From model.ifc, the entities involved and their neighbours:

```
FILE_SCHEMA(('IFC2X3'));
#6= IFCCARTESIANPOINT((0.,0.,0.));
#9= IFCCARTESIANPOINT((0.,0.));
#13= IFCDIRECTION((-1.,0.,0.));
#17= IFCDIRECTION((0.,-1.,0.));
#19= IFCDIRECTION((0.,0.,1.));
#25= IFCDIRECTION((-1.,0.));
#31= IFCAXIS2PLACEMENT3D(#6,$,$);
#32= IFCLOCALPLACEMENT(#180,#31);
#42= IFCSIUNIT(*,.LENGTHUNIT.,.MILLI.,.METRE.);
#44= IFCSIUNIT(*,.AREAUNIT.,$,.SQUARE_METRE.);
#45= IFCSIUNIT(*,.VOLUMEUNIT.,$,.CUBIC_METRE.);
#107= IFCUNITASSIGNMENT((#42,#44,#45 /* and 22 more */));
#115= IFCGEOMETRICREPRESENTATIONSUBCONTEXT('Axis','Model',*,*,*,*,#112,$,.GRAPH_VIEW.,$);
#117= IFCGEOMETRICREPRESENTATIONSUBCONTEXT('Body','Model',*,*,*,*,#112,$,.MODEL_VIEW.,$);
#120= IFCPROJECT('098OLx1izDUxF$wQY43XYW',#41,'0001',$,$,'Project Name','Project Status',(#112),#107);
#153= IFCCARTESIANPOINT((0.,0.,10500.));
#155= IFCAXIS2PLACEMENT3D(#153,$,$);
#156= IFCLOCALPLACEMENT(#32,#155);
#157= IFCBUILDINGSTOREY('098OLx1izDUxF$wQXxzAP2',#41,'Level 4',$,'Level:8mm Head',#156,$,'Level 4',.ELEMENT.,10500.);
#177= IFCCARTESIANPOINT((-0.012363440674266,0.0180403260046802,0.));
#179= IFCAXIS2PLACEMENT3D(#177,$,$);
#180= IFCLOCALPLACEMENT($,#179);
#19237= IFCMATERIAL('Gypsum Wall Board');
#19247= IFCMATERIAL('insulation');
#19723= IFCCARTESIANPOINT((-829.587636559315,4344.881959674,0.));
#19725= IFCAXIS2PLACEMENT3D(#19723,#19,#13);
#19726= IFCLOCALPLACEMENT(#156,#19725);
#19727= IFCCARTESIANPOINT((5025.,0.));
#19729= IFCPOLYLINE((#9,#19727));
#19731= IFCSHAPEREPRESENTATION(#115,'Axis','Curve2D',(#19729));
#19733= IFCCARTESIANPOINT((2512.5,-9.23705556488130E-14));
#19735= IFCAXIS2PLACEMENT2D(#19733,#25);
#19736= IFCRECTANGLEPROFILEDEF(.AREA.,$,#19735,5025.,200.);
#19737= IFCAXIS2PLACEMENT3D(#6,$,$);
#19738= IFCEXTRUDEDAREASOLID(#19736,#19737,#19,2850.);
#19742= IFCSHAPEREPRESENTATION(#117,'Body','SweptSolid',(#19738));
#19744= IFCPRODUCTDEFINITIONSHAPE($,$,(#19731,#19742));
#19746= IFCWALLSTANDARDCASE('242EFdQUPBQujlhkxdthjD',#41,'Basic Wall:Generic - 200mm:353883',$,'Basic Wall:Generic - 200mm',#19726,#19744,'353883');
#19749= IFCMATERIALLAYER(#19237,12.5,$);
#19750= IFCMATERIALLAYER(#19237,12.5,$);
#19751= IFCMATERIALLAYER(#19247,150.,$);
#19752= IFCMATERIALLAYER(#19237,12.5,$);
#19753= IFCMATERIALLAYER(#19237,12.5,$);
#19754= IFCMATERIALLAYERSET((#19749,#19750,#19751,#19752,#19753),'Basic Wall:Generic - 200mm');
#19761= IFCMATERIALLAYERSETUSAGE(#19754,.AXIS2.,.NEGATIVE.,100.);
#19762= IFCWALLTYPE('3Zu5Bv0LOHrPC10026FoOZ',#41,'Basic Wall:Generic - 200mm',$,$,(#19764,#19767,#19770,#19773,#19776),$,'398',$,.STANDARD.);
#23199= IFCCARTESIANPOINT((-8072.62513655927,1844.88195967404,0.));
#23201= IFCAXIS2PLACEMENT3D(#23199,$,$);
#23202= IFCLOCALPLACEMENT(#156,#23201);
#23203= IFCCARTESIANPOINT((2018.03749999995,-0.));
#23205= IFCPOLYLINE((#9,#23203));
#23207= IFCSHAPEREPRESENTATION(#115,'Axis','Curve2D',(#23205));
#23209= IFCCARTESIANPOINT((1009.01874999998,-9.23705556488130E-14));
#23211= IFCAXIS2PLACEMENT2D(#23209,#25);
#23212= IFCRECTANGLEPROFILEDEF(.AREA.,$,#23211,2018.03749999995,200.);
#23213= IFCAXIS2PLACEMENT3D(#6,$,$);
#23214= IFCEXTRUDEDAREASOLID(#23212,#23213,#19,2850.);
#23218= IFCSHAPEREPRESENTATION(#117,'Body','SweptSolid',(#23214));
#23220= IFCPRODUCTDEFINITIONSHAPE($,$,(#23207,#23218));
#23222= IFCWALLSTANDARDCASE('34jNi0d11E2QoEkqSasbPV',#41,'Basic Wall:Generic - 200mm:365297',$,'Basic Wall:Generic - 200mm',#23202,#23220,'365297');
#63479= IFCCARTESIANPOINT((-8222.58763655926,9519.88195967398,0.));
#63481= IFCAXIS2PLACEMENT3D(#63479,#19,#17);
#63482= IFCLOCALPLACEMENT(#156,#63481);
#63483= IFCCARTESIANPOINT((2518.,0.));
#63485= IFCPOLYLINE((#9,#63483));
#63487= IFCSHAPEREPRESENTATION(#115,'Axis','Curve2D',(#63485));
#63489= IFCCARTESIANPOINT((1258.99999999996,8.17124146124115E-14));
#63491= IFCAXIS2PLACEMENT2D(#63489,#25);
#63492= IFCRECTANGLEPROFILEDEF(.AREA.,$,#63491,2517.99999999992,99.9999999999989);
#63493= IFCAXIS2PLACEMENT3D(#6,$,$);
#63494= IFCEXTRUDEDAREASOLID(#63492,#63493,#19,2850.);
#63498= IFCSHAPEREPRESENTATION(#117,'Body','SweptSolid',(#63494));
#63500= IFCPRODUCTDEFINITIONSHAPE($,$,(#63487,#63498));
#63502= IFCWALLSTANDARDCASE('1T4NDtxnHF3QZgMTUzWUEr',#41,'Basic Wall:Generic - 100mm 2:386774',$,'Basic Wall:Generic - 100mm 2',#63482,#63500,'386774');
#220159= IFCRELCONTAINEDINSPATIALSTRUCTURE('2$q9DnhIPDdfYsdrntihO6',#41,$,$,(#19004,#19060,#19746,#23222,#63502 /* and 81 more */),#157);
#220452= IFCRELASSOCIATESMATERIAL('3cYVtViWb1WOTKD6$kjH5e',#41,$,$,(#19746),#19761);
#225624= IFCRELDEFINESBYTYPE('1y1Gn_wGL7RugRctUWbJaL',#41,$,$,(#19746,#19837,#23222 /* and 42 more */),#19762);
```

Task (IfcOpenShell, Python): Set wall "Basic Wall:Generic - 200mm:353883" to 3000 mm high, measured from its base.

```python
import ifcopenshell
import ifcopenshell.geom
import ifcopenshell.util.representation
import ifcopenshell.util.shape

model = ifcopenshell.open("model.ifc")
settings = ifcopenshell.geom.settings()


def volume(element):
    """Net volume in cubic metres, openings subtracted."""
    shape = ifcopenshell.geom.create_shape(settings, element)
    return ifcopenshell.util.shape.get_volume(shape.geometry)


wall = model.by_guid("242EFdQUPBQujlhkxdthjD")
before = volume(wall)

body = ifcopenshell.util.representation.get_representation(wall, "Model", "Body")
solid = body.Items[0]
old_height = solid.Depth
solid.Depth = 3000.0
after = volume(wall)

print(f"height {old_height:g} -> {solid.Depth:g}, volume {before:.3f} -> {after:.3f} m3")

model.write("model-out.ifc")
```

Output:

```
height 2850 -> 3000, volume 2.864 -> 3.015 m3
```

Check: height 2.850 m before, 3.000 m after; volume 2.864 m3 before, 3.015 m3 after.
